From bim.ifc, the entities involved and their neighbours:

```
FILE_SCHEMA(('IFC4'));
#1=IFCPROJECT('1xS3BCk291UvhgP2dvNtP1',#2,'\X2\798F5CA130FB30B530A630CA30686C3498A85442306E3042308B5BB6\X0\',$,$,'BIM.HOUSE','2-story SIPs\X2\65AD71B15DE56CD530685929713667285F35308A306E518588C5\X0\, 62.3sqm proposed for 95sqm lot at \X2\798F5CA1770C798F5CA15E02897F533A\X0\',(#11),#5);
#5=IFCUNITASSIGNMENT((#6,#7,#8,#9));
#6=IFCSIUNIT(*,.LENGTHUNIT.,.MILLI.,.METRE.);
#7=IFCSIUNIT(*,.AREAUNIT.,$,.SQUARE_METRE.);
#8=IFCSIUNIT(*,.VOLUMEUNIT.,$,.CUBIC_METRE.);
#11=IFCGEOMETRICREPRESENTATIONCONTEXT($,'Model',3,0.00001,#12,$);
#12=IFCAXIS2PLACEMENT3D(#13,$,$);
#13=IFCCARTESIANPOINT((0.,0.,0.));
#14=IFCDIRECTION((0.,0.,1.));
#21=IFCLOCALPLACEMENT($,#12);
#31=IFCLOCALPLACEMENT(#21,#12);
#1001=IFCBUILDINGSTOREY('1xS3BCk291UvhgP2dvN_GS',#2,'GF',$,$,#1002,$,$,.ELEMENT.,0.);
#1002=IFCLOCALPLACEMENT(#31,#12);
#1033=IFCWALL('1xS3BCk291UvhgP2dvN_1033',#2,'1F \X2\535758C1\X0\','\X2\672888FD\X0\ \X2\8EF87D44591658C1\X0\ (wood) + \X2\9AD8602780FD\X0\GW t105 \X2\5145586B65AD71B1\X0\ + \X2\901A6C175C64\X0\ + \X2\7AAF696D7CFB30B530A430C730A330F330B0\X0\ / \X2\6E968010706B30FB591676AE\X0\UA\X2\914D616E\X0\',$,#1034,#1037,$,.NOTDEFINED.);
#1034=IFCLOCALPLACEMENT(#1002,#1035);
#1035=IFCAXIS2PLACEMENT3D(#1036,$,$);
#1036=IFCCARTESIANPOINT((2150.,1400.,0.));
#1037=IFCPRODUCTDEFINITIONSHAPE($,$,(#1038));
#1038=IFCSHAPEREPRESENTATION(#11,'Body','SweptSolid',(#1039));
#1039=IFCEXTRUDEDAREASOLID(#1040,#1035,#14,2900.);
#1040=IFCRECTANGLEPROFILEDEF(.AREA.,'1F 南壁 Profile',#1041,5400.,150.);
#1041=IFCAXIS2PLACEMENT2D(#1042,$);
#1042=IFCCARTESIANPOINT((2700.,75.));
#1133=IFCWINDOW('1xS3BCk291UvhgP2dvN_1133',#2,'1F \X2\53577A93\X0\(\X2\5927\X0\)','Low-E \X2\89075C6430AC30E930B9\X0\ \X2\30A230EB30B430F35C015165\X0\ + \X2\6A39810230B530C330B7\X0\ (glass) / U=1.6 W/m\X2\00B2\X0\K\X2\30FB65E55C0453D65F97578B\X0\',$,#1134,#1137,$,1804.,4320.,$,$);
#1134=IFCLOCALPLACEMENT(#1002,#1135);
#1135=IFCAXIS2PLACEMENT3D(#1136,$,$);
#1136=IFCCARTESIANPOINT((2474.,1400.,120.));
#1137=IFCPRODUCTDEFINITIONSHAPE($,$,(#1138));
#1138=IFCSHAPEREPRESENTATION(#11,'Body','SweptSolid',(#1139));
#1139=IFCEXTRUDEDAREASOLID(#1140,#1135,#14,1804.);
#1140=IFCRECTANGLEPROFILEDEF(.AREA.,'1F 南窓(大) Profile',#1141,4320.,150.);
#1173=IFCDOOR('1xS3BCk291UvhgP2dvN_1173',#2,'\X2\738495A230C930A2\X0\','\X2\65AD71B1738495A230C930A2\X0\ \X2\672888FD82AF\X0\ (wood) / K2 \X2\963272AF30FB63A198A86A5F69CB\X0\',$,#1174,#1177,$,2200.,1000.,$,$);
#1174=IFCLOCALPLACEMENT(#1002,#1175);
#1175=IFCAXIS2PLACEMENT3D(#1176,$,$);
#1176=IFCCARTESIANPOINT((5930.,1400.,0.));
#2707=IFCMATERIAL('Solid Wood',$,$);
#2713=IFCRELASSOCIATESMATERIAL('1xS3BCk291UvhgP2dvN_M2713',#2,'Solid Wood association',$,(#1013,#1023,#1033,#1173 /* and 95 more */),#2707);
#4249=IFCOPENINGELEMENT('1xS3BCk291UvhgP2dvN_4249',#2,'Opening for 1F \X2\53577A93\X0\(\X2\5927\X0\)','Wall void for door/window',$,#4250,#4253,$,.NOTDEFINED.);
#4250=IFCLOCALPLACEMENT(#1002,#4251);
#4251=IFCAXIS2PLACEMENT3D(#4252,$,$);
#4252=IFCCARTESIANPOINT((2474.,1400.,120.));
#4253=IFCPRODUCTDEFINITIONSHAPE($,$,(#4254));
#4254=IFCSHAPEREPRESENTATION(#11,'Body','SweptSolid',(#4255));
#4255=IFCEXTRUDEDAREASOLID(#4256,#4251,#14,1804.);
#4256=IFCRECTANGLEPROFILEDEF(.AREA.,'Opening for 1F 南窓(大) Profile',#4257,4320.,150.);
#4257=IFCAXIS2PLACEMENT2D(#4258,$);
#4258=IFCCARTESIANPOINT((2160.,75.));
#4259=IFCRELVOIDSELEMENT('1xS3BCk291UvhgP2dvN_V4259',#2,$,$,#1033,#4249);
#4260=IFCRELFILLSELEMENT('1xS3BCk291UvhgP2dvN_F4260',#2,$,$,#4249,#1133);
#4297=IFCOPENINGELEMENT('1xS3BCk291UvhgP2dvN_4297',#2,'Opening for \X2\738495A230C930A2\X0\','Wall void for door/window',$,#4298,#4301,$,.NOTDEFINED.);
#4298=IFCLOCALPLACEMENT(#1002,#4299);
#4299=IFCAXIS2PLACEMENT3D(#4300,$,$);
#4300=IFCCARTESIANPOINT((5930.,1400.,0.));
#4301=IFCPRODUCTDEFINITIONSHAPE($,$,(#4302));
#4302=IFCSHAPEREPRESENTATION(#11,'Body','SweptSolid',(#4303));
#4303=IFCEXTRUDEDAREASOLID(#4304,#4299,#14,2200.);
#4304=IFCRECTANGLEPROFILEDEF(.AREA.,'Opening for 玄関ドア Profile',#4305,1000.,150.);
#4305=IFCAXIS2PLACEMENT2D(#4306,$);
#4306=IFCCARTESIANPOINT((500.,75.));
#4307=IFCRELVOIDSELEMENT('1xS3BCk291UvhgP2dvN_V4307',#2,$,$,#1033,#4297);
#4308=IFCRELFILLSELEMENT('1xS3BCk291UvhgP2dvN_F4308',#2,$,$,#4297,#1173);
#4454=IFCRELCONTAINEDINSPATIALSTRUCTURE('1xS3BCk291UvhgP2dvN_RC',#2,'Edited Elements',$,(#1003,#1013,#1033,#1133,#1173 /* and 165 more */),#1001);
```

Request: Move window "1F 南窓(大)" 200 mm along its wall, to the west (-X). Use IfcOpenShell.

```python
import ifcopenshell
import ifcopenshell.api.geometry
import ifcopenshell.util.placement
import ifcopenshell.util.unit

model = ifcopenshell.open("bim.ifc")
unit_scale = ifcopenshell.util.unit.calculate_unit_scale(model)

window = model.by_guid("1xS3BCk291UvhgP2dvN_1133")
opening = window.FillsVoids[0].RelatingOpeningElement
wall = opening.VoidsElements[0].RelatingBuildingElement

wall_matrix = ifcopenshell.util.placement.get_local_placement(wall.ObjectPlacement)
shift = wall_matrix[:3, 0] * -0.2 / unit_scale
before = ifcopenshell.util.placement.get_local_placement(window.ObjectPlacement)[:3, 3].copy()

# The window is not placed relative to its opening, so move both.
for product in (opening, window):
    matrix = ifcopenshell.util.placement.get_local_placement(product.ObjectPlacement)
    matrix[:3, 3] += shift
    ifcopenshell.api.geometry.edit_object_placement(model, product=product, matrix=matrix, is_si=False)

after = ifcopenshell.util.placement.get_local_placement(window.ObjectPlacement)[:3, 3]
print("window moved by", (after - before).round(3) + 0.0)

model.write("bim-out.ifc")
```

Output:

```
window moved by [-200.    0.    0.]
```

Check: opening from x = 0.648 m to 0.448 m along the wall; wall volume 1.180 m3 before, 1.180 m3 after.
